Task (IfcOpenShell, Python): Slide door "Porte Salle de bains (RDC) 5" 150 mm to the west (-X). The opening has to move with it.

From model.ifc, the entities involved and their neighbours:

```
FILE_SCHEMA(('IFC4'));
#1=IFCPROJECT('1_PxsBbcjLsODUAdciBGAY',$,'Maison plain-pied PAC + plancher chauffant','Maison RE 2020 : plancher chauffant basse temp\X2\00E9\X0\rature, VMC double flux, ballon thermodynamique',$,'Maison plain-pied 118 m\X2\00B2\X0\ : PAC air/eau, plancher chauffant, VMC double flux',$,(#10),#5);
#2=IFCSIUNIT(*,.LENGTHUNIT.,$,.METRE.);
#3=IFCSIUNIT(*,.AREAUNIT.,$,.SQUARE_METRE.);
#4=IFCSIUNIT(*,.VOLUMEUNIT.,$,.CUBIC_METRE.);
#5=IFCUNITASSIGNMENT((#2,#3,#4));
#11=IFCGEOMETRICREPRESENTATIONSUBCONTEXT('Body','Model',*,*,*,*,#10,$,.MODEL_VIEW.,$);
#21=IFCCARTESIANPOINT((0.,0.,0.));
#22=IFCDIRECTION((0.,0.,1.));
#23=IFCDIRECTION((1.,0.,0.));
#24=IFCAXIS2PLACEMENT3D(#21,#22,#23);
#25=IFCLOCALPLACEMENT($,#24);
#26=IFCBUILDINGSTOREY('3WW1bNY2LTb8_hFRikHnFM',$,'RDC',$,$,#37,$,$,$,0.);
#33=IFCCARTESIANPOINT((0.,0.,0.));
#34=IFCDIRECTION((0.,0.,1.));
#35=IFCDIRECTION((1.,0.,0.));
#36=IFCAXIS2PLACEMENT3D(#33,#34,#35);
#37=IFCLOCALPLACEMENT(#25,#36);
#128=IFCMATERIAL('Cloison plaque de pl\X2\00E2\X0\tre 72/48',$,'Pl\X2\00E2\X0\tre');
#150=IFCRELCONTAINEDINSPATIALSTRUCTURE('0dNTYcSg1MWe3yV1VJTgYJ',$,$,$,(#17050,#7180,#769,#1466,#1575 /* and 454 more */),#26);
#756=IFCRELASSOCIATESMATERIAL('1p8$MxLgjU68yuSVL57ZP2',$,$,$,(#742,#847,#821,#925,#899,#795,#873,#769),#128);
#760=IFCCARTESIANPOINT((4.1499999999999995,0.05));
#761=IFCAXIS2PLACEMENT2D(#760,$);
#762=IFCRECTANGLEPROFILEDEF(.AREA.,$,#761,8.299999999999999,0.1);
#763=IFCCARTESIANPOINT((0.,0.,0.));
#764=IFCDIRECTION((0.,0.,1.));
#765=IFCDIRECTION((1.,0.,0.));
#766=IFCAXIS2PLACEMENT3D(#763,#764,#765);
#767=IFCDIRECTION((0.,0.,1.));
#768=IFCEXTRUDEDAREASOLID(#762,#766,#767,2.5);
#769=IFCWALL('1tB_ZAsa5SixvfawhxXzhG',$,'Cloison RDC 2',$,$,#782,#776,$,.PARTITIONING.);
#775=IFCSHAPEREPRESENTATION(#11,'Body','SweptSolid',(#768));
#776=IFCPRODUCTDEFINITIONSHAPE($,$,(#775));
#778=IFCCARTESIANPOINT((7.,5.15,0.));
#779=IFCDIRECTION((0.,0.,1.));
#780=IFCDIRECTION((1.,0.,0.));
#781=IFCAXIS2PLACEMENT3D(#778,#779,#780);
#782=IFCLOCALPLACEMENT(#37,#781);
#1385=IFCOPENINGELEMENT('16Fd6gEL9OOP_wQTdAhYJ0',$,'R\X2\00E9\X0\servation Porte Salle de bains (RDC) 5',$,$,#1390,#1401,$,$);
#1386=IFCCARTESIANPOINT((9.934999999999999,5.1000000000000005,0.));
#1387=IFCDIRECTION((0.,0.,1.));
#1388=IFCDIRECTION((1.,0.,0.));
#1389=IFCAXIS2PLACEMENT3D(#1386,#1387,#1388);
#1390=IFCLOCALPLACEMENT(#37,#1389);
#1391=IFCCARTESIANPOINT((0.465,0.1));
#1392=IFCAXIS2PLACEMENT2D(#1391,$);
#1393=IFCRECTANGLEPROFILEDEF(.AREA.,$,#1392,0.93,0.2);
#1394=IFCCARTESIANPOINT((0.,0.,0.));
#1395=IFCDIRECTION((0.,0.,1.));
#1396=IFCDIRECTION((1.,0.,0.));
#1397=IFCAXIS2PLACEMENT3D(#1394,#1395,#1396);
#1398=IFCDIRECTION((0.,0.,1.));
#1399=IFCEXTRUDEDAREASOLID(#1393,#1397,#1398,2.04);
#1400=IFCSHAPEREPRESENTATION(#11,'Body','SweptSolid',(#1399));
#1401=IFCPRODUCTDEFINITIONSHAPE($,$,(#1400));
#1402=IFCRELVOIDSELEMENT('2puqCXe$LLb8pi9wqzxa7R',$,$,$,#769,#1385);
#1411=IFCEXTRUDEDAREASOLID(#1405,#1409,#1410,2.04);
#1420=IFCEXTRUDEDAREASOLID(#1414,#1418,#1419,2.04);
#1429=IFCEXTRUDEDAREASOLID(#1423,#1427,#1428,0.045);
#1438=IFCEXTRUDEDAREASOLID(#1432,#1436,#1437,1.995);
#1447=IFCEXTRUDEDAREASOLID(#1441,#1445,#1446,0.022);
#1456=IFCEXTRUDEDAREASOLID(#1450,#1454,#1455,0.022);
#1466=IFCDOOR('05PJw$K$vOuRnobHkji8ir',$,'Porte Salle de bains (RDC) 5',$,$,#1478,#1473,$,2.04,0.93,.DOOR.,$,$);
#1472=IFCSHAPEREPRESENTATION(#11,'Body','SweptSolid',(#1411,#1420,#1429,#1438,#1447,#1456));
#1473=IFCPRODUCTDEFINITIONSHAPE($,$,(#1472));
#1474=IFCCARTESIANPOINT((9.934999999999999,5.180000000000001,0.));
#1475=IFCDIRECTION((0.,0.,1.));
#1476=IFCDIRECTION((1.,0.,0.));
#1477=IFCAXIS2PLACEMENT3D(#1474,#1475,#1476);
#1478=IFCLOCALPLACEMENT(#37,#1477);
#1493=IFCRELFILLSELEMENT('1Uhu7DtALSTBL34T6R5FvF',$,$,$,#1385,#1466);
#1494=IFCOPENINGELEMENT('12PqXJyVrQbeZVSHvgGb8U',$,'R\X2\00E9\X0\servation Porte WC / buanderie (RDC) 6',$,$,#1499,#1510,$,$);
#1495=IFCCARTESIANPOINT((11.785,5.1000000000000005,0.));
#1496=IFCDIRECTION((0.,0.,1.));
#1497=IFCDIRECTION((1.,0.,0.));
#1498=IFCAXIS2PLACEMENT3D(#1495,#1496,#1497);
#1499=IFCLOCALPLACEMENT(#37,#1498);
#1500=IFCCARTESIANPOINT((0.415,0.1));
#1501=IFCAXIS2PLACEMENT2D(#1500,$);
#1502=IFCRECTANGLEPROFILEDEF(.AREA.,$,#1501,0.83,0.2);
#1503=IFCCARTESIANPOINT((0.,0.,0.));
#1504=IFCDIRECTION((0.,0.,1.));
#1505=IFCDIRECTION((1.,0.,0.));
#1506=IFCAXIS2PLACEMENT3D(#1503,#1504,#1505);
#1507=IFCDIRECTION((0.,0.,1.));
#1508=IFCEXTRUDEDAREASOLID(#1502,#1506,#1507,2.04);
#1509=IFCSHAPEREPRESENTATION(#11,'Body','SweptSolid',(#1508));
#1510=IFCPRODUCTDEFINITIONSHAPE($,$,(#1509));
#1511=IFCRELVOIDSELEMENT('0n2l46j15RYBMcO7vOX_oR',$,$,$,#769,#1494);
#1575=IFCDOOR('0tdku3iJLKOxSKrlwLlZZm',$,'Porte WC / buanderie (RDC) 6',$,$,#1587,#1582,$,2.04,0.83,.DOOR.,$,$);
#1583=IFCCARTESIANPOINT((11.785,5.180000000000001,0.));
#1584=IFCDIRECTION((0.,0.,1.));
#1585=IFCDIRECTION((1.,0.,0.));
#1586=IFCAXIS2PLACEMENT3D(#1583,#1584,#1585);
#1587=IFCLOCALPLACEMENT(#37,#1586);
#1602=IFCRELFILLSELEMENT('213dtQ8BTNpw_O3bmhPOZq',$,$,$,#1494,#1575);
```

```python
import ifcopenshell
import ifcopenshell.api.geometry
import ifcopenshell.util.placement

model = ifcopenshell.open("model.ifc")

door = model.by_guid("05PJw$K$vOuRnobHkji8ir")
opening = door.FillsVoids[0].RelatingOpeningElement
wall = opening.VoidsElements[0].RelatingBuildingElement

wall_matrix = ifcopenshell.util.placement.get_local_placement(wall.ObjectPlacement)
shift = wall_matrix[:3, 0] * -0.15
before = ifcopenshell.util.placement.get_local_placement(door.ObjectPlacement)[:3, 3].copy()

# The door is not placed relative to its opening, so move both.
for product in (opening, door):
    matrix = ifcopenshell.util.placement.get_local_placement(product.ObjectPlacement)
    matrix[:3, 3] += shift
    ifcopenshell.api.geometry.edit_object_placement(model, product=product, matrix=matrix, is_si=False)

after = ifcopenshell.util.placement.get_local_placement(door.ObjectPlacement)[:3, 3]
print("door moved by", (after - before).round(3) + 0.0)

model.write("model-out.ifc")
```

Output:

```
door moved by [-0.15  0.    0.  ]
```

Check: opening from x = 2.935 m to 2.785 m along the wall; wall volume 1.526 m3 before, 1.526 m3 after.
